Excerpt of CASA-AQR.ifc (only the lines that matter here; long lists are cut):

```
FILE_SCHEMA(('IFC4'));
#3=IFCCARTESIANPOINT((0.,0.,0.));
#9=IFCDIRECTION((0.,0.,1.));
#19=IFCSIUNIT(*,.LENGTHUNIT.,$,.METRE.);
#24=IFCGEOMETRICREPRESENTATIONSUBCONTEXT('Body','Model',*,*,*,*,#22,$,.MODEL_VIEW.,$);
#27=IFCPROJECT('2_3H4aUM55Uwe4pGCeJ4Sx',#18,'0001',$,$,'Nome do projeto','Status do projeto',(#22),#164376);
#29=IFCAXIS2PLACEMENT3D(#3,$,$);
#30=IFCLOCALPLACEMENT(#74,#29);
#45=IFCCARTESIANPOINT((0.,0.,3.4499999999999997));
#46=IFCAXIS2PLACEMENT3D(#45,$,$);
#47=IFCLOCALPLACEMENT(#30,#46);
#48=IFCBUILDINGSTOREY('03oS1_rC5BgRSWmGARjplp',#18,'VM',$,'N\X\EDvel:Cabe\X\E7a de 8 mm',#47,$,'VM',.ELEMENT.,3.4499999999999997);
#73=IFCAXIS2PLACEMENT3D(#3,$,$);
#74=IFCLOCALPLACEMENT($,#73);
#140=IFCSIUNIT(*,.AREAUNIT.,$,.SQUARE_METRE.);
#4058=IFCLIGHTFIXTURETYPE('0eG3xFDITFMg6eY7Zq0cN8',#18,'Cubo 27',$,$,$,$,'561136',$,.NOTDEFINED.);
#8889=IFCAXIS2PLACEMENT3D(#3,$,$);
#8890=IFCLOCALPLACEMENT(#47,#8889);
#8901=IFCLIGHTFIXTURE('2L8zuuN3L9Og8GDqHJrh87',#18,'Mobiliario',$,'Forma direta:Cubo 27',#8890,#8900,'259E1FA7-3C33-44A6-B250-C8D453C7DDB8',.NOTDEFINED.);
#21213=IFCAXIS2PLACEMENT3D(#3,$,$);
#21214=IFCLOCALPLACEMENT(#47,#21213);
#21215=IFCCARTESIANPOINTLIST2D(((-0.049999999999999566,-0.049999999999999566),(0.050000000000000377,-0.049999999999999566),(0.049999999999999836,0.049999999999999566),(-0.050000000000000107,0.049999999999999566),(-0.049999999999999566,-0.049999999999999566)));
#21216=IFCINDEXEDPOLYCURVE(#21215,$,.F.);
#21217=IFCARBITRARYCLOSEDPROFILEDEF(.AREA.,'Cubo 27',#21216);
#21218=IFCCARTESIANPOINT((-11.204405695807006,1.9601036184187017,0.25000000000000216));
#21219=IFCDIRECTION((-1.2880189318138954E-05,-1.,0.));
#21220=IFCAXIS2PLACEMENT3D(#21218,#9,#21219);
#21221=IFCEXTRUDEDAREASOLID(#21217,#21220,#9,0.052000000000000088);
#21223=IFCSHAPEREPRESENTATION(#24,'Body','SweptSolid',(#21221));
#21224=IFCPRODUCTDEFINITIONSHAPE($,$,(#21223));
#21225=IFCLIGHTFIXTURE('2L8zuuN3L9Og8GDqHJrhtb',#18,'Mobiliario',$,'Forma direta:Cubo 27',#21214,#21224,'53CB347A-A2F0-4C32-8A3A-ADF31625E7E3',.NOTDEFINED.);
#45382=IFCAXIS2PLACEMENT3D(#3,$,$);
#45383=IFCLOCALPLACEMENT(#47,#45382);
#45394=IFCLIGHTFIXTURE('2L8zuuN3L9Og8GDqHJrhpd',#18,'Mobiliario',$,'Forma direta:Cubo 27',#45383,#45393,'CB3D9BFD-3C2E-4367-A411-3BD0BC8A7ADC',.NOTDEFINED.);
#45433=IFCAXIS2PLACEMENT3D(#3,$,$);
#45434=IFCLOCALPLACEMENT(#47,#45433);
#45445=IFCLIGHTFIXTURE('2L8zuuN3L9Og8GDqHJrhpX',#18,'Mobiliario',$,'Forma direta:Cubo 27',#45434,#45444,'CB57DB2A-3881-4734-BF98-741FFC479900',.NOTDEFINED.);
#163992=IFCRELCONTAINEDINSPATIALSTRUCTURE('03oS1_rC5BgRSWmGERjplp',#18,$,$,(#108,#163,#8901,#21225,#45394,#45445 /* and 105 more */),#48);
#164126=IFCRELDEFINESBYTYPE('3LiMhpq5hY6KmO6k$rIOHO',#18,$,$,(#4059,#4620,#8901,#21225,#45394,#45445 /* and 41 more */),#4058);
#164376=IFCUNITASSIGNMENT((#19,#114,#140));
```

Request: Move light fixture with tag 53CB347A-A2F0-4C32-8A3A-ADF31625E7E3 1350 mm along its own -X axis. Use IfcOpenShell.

```python
import ifcopenshell
import ifcopenshell.api.geometry
import ifcopenshell.util.placement

model = ifcopenshell.open("CASA-AQR.ifc")

item = model.by_guid("2L8zuuN3L9Og8GDqHJrhtb")
matrix = ifcopenshell.util.placement.get_local_placement(item.ObjectPlacement)
matrix[:3, 3] -= matrix[:3, 0] * 1.35
ifcopenshell.api.geometry.edit_object_placement(model, product=item, matrix=matrix, is_si=False)

print(ifcopenshell.util.placement.get_local_placement(item.ObjectPlacement).round(3) + 0.0)

model.write("CASA-AQR_edited.ifc")
```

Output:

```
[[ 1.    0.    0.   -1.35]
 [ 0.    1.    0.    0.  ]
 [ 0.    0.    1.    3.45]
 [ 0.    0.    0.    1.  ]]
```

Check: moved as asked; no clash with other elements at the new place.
